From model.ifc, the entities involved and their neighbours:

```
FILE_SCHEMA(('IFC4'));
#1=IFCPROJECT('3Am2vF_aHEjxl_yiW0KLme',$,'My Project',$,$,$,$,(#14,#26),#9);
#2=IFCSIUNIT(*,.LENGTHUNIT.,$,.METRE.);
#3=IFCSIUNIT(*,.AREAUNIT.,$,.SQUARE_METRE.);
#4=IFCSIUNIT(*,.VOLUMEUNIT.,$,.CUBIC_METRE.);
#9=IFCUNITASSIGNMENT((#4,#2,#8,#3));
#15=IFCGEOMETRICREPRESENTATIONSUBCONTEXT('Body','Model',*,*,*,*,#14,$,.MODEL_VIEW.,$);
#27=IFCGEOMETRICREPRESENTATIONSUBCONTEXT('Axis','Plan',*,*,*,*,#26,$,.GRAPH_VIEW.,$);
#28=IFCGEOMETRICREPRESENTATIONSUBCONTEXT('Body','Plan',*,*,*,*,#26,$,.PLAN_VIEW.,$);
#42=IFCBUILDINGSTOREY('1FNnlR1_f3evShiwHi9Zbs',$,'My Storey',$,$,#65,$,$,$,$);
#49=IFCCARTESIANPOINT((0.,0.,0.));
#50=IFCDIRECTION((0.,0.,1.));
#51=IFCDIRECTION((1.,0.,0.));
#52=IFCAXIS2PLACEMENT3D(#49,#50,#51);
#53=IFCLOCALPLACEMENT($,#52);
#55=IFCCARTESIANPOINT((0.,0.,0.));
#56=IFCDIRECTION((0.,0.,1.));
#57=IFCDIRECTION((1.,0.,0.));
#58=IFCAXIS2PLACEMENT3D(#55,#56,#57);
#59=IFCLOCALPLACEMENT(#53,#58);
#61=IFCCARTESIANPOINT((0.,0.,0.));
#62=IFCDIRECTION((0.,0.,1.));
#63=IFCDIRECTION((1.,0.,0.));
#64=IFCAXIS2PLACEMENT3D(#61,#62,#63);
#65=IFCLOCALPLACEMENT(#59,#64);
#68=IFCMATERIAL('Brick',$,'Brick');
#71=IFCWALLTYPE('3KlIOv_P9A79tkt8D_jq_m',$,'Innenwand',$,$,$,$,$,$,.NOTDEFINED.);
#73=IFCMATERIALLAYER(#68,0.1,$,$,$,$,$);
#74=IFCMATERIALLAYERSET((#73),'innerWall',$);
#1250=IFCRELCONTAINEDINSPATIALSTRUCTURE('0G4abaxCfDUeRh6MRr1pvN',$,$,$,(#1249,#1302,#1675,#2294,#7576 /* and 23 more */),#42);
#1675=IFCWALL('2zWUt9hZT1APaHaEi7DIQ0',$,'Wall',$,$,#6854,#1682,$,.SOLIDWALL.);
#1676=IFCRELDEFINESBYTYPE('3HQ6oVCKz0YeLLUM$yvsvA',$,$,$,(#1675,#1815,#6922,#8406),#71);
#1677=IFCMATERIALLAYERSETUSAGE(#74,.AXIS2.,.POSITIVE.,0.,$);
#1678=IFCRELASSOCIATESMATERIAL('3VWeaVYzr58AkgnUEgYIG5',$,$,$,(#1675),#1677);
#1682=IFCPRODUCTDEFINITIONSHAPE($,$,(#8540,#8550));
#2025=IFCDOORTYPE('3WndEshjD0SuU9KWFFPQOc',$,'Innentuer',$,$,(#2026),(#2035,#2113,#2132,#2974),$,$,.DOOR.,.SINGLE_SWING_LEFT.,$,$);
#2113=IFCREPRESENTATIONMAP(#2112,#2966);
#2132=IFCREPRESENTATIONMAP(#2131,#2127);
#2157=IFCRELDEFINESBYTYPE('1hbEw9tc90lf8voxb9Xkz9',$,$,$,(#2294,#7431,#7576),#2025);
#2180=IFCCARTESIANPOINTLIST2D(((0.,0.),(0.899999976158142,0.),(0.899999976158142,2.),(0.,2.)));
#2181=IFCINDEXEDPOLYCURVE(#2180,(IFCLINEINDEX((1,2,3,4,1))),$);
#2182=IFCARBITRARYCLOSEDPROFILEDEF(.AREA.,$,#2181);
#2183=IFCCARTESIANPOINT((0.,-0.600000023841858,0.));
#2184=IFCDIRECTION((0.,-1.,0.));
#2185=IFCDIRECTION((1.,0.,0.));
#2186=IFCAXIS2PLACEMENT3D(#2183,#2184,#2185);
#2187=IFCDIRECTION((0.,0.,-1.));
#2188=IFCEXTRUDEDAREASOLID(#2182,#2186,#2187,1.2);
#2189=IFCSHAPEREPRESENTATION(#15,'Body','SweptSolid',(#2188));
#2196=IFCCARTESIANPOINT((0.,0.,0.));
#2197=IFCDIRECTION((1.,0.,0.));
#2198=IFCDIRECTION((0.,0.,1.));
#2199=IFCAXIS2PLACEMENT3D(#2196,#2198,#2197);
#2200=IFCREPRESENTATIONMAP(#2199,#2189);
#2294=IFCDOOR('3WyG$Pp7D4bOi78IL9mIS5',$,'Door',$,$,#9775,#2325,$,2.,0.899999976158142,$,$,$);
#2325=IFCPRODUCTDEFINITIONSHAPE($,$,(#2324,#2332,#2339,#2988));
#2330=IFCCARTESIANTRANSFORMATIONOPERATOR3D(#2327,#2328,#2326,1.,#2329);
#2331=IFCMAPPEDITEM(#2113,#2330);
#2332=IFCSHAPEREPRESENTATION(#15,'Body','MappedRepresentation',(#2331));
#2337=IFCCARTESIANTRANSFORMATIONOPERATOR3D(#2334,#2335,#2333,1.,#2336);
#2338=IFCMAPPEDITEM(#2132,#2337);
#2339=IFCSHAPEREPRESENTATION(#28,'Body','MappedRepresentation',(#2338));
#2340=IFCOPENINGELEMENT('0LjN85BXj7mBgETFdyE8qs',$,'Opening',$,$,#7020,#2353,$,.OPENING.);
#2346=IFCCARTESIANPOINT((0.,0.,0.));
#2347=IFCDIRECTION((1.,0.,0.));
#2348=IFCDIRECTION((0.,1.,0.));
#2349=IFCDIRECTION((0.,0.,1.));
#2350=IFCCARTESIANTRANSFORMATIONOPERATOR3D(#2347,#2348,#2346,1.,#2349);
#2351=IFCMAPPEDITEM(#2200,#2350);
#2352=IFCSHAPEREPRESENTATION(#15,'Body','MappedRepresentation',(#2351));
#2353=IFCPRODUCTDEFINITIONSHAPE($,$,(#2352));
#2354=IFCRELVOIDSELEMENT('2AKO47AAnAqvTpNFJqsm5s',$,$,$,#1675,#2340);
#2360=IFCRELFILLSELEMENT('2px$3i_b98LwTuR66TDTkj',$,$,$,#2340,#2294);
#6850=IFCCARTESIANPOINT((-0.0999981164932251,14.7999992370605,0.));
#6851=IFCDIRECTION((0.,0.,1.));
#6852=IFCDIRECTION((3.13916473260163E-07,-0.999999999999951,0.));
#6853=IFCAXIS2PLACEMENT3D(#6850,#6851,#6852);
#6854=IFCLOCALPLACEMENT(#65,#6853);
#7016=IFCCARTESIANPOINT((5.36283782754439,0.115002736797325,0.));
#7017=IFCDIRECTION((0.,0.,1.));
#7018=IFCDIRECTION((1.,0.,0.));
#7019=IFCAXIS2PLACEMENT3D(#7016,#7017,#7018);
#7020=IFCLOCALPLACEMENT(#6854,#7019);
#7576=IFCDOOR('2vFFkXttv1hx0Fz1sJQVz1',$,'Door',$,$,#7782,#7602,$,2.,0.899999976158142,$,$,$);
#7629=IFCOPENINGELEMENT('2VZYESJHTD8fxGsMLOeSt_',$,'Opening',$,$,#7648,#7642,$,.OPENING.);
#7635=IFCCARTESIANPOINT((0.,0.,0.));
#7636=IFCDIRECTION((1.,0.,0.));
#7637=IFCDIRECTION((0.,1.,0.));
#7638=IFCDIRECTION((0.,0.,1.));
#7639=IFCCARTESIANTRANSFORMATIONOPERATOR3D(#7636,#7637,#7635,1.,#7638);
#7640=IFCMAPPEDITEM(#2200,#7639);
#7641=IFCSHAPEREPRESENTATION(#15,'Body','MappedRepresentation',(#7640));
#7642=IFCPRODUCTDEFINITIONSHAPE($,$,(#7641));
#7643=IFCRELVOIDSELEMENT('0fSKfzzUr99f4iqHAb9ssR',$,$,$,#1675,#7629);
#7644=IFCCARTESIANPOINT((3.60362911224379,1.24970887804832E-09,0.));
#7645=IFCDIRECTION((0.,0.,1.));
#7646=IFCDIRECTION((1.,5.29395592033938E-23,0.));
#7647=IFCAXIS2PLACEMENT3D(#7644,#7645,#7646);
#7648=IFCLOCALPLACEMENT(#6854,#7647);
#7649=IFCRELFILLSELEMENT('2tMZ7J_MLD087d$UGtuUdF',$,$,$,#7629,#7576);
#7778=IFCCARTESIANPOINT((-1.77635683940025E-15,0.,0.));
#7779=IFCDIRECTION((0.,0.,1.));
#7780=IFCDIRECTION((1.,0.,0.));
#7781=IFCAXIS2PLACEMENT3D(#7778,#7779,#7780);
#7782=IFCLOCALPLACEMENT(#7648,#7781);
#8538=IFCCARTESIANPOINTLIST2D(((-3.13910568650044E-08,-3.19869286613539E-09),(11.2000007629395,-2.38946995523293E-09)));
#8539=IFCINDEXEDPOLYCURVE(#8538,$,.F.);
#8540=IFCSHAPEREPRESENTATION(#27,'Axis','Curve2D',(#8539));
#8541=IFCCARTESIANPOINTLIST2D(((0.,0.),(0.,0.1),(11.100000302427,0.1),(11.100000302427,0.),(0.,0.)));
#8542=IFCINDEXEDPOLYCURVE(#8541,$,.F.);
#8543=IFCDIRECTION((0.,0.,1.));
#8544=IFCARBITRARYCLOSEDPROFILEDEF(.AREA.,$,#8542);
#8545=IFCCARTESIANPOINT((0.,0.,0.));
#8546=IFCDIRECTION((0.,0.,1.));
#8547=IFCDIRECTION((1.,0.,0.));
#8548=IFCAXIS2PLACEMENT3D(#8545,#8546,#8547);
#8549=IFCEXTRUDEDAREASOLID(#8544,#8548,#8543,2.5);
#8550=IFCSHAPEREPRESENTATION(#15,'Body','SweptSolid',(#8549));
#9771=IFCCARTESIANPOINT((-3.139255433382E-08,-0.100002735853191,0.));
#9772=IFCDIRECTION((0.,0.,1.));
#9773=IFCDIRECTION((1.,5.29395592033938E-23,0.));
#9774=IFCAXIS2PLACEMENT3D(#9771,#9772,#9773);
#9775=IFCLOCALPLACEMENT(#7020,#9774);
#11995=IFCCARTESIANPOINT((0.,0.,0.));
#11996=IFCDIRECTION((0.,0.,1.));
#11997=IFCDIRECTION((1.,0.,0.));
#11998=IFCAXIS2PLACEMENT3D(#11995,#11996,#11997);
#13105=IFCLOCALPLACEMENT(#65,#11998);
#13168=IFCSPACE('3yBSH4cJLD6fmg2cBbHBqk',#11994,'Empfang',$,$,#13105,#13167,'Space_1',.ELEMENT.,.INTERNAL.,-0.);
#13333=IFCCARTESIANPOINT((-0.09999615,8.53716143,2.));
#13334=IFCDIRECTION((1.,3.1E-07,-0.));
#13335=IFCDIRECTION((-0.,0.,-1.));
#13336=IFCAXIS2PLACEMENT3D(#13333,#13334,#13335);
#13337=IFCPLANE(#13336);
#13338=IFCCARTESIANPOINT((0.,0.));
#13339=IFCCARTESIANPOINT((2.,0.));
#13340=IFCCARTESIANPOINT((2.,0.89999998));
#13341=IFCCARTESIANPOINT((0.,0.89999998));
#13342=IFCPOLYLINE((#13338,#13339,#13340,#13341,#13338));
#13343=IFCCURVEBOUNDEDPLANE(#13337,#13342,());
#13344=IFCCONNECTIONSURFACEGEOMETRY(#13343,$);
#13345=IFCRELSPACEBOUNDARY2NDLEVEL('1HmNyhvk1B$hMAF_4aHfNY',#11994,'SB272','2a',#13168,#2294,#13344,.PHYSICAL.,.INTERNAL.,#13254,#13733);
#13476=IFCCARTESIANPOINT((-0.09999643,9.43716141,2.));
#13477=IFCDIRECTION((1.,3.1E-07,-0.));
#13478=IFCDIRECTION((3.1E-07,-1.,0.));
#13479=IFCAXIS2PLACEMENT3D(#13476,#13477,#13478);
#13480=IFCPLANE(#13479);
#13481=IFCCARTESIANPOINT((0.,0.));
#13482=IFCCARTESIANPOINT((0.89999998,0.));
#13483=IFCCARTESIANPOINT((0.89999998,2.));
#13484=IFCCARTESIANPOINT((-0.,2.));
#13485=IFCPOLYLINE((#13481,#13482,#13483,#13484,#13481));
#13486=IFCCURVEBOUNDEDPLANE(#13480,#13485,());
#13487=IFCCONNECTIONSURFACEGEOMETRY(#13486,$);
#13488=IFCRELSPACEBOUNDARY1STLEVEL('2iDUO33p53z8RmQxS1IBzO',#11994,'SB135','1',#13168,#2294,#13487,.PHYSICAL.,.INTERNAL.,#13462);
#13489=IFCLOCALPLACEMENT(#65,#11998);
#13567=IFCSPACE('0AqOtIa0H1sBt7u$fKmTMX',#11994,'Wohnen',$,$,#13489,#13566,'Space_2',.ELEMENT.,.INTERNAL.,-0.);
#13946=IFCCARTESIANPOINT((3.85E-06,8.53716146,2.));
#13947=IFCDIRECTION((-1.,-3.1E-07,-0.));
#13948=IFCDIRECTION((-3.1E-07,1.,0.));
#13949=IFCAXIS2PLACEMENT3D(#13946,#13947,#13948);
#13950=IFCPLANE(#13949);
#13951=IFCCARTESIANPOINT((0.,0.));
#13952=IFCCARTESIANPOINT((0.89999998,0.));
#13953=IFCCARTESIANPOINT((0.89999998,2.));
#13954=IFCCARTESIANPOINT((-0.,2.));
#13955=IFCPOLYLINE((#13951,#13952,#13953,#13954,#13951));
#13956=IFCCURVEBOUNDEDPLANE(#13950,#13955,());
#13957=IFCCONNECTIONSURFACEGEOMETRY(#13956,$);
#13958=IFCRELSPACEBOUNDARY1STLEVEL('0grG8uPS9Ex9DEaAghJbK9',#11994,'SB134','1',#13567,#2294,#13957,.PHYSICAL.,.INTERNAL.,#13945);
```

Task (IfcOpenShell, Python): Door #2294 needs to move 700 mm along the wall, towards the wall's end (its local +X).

```python
import numpy as np
import ifcopenshell
import ifcopenshell.api.geometry
import ifcopenshell.util.placement
import ifcopenshell.util.unit

model = ifcopenshell.open("model.ifc")
unit_scale = ifcopenshell.util.unit.calculate_unit_scale(model)

door = model.by_guid("3WyG$Pp7D4bOi78IL9mIS5")
opening = door.FillsVoids[0].RelatingOpeningElement
wall = opening.VoidsElements[0].RelatingBuildingElement

wall_matrix = ifcopenshell.util.placement.get_local_placement(wall.ObjectPlacement)
shift = wall_matrix[:3, 0] * 0.7 / unit_scale
before = ifcopenshell.util.placement.get_local_placement(door.ObjectPlacement)[:3, 3].copy()

# The door is placed relative to its opening, so it follows when the opening moves.
matrix = ifcopenshell.util.placement.get_local_placement(opening.ObjectPlacement)
matrix[:3, 3] += shift
ifcopenshell.api.geometry.edit_object_placement(
    model, product=opening, matrix=matrix, is_si=False, should_transform_children=True
)

# Space boundary surfaces are stored in each space's coordinates; move them too.
for rel in door.ProvidesBoundaries:
    if not rel.ConnectionGeometry:
        continue
    surface = rel.ConnectionGeometry.SurfaceOnRelatingElement.BasisSurface
    space_matrix = ifcopenshell.util.placement.get_local_placement(rel.RelatingSpace.ObjectPlacement)
    point = np.array(surface.Position.Location.Coordinates) + space_matrix[:3, :3].T @ shift
    surface.Position = model.createIfcAxis2Placement3D(
        model.createIfcCartesianPoint(point.tolist()), surface.Position.Axis, surface.Position.RefDirection
    )

after = ifcopenshell.util.placement.get_local_placement(door.ObjectPlacement)[:3, 3]
print("door moved by", (after - before).round(3) + 0.0)

model.write("model_edited.ifc")
```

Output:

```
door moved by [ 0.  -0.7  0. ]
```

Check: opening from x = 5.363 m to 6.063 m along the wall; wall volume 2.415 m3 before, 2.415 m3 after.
